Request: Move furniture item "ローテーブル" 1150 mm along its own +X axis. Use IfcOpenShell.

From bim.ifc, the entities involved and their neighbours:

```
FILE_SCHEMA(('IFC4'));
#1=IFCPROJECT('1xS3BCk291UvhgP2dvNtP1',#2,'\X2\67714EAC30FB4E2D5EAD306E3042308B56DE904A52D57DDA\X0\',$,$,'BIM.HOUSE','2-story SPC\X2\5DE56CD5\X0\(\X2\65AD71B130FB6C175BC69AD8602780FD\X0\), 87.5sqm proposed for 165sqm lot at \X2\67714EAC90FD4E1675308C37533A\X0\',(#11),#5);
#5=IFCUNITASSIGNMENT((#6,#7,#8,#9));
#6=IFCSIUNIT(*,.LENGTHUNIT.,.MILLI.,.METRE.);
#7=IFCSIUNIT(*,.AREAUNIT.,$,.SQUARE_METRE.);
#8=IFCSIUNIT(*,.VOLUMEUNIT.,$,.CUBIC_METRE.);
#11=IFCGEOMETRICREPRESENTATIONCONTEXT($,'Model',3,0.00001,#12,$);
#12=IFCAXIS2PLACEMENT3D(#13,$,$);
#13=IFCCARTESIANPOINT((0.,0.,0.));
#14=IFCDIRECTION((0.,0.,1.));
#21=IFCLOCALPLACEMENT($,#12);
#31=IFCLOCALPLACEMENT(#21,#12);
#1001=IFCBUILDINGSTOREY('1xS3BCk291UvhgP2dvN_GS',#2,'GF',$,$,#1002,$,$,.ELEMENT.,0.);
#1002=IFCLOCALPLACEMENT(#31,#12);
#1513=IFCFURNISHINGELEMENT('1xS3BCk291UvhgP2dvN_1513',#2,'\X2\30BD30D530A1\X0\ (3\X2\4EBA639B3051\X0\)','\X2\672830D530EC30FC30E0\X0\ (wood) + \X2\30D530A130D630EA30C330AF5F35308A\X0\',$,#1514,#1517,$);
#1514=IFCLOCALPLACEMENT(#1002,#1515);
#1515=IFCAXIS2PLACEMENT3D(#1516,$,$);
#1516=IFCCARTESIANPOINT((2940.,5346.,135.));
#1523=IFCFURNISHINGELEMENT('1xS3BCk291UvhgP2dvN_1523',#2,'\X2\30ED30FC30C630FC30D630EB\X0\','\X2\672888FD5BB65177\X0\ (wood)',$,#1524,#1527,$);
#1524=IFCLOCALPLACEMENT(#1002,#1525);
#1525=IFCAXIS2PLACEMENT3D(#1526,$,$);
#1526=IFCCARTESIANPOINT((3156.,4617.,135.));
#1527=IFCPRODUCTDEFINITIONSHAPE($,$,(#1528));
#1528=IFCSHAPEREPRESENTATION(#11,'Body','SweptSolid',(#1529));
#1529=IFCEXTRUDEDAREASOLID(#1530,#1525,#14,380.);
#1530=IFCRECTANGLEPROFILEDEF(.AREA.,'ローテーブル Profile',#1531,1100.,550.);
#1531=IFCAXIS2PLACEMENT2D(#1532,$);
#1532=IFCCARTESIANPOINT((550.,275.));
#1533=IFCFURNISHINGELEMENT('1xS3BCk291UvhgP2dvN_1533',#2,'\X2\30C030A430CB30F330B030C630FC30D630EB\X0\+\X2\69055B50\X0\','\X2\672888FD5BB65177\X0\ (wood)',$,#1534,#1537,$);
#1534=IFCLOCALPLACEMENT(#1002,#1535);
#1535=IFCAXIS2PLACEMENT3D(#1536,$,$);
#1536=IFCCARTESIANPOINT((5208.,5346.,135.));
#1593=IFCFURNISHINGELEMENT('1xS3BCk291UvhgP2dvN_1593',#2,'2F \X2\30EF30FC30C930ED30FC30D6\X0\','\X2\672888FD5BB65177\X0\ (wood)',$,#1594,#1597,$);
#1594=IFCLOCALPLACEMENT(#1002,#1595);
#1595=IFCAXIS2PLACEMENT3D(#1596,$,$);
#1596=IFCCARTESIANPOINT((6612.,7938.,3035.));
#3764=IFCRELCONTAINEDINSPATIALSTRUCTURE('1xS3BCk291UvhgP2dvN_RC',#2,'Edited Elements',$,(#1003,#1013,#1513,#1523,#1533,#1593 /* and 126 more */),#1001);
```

```python
import ifcopenshell
import ifcopenshell.api.geometry
import ifcopenshell.util.placement
import ifcopenshell.util.unit

model = ifcopenshell.open("bim.ifc")
unit_scale = ifcopenshell.util.unit.calculate_unit_scale(model)

item = model.by_id(1523)
matrix = ifcopenshell.util.placement.get_local_placement(item.ObjectPlacement)
matrix[:3, 3] += matrix[:3, 0] * 1.15 / unit_scale
ifcopenshell.api.geometry.edit_object_placement(model, product=item, matrix=matrix, is_si=False)

print(ifcopenshell.util.placement.get_local_placement(item.ObjectPlacement).round(3) + 0.0)

model.write("bim_updated.ifc")
```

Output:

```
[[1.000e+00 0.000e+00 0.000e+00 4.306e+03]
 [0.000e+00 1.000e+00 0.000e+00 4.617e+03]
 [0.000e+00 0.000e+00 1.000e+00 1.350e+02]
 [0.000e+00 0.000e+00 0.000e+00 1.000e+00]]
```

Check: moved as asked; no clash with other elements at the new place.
